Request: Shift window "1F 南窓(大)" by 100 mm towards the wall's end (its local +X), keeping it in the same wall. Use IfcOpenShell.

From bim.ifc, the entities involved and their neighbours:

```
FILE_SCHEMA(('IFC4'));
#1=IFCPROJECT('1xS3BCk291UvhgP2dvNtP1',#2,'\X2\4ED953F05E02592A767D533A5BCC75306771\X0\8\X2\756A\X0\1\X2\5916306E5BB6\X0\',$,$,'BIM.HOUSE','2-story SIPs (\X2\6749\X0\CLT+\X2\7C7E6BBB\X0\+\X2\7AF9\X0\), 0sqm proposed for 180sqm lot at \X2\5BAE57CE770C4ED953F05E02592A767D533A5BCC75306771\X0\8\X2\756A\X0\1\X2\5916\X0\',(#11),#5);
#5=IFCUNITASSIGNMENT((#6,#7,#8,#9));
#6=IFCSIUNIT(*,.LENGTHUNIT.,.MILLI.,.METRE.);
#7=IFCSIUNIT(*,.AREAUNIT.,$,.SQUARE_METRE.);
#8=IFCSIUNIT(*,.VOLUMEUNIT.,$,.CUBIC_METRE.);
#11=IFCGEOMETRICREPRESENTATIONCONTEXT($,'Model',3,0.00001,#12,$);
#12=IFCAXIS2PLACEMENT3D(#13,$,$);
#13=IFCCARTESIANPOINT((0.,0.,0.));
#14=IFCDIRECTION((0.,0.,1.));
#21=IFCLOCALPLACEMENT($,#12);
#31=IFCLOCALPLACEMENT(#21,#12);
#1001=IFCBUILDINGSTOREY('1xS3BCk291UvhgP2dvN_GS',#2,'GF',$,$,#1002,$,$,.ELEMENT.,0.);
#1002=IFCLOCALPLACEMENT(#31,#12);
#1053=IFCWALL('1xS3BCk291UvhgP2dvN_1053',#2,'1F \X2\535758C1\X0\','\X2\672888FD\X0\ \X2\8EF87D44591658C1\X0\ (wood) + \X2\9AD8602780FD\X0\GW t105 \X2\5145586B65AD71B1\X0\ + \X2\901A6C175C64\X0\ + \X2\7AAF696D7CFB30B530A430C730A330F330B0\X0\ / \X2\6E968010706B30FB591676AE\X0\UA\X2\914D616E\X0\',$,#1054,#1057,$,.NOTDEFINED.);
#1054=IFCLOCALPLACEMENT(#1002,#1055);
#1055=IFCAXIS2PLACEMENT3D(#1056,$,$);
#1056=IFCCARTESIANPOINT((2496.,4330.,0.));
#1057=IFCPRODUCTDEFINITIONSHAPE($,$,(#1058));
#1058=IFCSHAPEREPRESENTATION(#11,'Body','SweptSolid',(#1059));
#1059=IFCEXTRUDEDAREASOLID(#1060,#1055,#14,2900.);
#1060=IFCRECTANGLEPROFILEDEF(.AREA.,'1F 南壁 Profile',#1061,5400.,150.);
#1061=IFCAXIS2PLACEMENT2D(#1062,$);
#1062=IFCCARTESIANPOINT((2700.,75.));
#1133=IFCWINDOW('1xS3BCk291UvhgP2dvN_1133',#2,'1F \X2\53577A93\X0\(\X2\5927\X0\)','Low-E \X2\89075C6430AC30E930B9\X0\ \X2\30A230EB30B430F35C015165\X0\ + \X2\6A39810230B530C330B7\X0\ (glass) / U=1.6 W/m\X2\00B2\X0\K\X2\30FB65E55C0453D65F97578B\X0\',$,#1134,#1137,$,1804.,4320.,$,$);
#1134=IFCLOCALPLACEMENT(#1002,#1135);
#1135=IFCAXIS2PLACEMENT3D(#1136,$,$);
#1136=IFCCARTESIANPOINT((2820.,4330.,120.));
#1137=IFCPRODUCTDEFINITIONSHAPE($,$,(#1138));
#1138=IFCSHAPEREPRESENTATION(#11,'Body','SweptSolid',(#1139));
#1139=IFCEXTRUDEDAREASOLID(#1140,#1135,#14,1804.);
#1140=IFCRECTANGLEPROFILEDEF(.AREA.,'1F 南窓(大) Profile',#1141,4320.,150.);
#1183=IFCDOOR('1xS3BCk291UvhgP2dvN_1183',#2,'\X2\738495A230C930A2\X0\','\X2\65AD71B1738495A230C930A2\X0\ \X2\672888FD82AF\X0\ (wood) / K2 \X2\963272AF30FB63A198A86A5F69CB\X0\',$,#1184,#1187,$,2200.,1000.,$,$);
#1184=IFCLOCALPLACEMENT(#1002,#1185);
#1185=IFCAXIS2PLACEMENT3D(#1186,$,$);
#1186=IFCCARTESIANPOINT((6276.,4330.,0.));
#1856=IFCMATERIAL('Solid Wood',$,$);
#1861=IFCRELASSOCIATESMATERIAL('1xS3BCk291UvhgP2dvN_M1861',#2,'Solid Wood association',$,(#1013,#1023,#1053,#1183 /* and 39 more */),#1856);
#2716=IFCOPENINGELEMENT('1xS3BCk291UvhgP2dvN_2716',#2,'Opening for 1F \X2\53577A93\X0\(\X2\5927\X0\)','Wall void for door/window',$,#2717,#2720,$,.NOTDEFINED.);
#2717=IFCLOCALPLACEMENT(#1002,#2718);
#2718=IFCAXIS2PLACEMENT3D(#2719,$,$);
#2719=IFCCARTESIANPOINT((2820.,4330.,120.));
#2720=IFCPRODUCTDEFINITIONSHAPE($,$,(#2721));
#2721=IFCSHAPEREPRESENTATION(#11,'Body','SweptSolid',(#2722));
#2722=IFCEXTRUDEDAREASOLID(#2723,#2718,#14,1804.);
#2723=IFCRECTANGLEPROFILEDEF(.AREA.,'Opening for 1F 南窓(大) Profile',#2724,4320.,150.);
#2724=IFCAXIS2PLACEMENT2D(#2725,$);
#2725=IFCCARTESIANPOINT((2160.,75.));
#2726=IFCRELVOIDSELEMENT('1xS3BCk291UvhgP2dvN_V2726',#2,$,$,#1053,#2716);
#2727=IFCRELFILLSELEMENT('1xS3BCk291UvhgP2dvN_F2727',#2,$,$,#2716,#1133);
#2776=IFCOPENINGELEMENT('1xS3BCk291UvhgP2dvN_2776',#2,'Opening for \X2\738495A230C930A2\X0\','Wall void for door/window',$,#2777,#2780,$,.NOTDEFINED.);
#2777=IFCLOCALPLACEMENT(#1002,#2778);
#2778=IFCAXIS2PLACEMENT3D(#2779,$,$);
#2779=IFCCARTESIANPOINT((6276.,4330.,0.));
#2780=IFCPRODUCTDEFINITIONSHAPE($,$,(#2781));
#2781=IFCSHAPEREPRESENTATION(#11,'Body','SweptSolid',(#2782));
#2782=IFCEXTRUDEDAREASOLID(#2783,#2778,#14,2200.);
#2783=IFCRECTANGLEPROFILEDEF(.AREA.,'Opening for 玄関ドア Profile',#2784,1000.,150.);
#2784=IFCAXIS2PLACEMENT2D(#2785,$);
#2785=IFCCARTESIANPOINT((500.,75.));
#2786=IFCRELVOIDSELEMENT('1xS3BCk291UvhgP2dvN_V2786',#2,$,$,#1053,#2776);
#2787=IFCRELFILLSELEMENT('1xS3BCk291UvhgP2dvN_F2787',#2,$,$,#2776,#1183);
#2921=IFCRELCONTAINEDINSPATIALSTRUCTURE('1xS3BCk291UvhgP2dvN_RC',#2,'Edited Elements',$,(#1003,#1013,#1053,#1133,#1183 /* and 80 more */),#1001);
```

```python
import ifcopenshell
import ifcopenshell.api.geometry
import ifcopenshell.util.placement
import ifcopenshell.util.unit

model = ifcopenshell.open("bim.ifc")
unit_scale = ifcopenshell.util.unit.calculate_unit_scale(model)

window = model.by_guid("1xS3BCk291UvhgP2dvN_1133")
opening = window.FillsVoids[0].RelatingOpeningElement
wall = opening.VoidsElements[0].RelatingBuildingElement

wall_matrix = ifcopenshell.util.placement.get_local_placement(wall.ObjectPlacement)
shift = wall_matrix[:3, 0] * 0.1 / unit_scale
before = ifcopenshell.util.placement.get_local_placement(window.ObjectPlacement)[:3, 3].copy()

# The window is not placed relative to its opening, so move both.
for product in (opening, window):
    matrix = ifcopenshell.util.placement.get_local_placement(product.ObjectPlacement)
    matrix[:3, 3] += shift
    ifcopenshell.api.geometry.edit_object_placement(model, product=product, matrix=matrix, is_si=False)

after = ifcopenshell.util.placement.get_local_placement(window.ObjectPlacement)[:3, 3]
print("window moved by", (after - before).round(3) + 0.0)

model.write("bim_v2.ifc")
```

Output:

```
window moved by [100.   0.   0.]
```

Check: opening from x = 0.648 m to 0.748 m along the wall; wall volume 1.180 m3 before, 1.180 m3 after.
